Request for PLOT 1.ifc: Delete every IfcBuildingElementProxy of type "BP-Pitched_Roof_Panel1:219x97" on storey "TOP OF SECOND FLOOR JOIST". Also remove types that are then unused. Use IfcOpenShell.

First a look at what the model holds.

```python
import ifcopenshell
import ifcopenshell.util.element

model = ifcopenshell.open("PLOT 1.ifc")
print(model.schema)
storey = next(s for s in model.by_type("IfcBuildingStorey") if s.Name == "TOP OF SECOND FLOOR JOIST")
proxies = [e for e in ifcopenshell.util.element.get_decomposition(storey) if e.is_a("IfcBuildingElementProxy")]
seen = {}
for e in proxies:
    element_type = ifcopenshell.util.element.get_type(e)
    name = element_type.Name if element_type not in (None, e) else None
    seen[name] = seen.get(name, 0) + 1
for name, count in sorted(seen.items(), key=str):
    print(count, "x", name)
```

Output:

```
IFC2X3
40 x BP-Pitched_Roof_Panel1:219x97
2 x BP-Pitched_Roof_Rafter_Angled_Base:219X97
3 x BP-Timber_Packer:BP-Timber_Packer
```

```python
import ifcopenshell
import ifcopenshell.api.root
import ifcopenshell.util.element

model = ifcopenshell.open("PLOT 1.ifc")

storey = next(s for s in model.by_type("IfcBuildingStorey") if s.Name == "TOP OF SECOND FLOOR JOIST")
proxies = [e for e in ifcopenshell.util.element.get_decomposition(storey) if e.is_a("IfcBuildingElementProxy")]
targets = [e for e in proxies if (t := ifcopenshell.util.element.get_type(e)) not in (None, e) and t.Name == "BP-Pitched_Roof_Panel1:219x97"]
types = {ifcopenshell.util.element.get_type(e) for e in targets} - {None, *targets}

for e in targets:
    ifcopenshell.api.root.remove_product(model, product=e)
print(len(targets), "removed")

unused = [t for t in types if not ifcopenshell.util.element.get_types(t)]
for t in unused:
    ifcopenshell.api.root.remove_product(model, product=t)
print(len(unused), "unused types removed")

model.write("PLOT 1_edited.ifc")
```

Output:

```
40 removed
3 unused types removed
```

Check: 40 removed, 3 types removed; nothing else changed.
